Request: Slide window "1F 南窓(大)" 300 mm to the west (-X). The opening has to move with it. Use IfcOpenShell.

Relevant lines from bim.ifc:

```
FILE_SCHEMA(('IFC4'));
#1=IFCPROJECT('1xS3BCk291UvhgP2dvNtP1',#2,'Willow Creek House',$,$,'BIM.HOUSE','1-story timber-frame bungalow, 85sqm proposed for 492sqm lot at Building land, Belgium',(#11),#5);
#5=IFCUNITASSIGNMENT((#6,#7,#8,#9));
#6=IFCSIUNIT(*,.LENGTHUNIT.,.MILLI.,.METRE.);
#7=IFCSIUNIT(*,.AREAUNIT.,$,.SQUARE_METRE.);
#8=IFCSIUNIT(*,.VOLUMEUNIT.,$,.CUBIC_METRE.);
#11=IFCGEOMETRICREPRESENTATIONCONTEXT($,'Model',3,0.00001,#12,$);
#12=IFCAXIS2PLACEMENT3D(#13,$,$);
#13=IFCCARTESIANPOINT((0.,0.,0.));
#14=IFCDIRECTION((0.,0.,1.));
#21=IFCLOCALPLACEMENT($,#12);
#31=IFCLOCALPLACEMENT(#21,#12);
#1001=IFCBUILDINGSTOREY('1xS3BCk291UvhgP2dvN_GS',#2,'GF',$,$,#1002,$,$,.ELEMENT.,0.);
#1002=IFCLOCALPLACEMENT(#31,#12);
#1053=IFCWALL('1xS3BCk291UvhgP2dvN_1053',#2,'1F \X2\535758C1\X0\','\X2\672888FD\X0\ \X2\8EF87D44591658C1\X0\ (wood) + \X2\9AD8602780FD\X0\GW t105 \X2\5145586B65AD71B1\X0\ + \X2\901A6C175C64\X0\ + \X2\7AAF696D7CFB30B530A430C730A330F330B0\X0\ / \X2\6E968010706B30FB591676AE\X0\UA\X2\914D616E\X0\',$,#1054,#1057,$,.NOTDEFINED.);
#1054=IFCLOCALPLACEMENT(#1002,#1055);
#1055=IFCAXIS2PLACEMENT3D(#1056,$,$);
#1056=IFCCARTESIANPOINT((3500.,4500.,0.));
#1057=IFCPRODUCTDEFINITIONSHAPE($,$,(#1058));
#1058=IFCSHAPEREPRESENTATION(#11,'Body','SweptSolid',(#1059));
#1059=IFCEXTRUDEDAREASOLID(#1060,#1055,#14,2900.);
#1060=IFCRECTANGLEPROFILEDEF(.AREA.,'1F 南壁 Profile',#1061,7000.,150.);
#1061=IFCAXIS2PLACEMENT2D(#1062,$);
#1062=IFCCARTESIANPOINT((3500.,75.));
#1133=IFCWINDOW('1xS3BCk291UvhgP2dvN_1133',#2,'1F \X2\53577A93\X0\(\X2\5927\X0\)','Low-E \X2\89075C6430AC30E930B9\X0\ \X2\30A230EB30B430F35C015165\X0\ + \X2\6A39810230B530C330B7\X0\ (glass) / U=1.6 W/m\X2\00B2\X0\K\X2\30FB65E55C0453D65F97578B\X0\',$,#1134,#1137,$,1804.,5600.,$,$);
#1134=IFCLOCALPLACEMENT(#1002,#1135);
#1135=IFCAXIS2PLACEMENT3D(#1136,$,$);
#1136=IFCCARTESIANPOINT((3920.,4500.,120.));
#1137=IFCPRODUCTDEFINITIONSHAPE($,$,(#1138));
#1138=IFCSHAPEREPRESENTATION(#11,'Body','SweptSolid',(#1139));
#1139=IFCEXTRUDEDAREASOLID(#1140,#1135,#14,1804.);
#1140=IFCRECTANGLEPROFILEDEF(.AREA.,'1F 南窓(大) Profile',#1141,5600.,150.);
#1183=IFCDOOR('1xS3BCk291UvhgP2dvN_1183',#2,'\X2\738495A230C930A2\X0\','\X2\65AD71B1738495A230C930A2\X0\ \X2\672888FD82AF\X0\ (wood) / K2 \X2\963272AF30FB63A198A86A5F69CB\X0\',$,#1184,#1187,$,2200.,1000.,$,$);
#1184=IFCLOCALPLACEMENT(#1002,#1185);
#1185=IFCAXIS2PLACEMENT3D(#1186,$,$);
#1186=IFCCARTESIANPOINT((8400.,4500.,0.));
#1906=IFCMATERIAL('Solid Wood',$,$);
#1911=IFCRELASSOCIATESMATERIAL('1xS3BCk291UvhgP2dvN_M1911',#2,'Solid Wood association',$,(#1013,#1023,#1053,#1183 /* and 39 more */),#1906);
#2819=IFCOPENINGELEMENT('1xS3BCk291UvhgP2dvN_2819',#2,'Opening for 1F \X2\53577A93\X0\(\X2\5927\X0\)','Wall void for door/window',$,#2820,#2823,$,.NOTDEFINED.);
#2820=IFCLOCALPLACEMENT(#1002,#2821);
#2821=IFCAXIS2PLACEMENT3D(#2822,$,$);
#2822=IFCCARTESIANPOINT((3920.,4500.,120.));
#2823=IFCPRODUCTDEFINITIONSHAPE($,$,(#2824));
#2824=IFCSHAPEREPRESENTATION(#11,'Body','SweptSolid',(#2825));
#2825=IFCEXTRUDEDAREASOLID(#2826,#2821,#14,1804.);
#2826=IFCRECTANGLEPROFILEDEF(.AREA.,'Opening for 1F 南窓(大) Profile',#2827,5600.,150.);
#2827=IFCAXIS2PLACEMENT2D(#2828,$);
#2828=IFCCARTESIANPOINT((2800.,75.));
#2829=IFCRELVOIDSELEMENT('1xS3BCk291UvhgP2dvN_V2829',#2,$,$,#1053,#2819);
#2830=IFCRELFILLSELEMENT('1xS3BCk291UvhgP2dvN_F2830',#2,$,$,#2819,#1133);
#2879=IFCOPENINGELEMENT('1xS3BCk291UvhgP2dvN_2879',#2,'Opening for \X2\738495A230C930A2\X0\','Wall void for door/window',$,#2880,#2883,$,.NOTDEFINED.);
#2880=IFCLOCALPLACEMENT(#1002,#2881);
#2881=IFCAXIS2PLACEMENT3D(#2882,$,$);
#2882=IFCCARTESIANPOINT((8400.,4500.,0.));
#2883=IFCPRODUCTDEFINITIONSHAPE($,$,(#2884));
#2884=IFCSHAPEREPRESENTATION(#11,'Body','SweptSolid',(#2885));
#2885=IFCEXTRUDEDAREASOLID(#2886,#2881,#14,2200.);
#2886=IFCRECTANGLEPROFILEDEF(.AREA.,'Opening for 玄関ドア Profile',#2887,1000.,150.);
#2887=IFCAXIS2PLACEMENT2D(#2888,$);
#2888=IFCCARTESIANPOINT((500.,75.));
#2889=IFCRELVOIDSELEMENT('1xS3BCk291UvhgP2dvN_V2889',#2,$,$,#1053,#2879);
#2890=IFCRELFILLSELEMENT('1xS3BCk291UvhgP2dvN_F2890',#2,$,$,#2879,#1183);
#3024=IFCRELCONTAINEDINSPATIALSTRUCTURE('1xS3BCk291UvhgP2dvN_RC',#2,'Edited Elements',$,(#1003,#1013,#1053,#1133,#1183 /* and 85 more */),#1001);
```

```python
import ifcopenshell
import ifcopenshell.api.geometry
import ifcopenshell.util.placement
import ifcopenshell.util.unit

model = ifcopenshell.open("bim.ifc")
unit_scale = ifcopenshell.util.unit.calculate_unit_scale(model)

window = model.by_guid("1xS3BCk291UvhgP2dvN_1133")
opening = window.FillsVoids[0].RelatingOpeningElement
wall = opening.VoidsElements[0].RelatingBuildingElement

wall_matrix = ifcopenshell.util.placement.get_local_placement(wall.ObjectPlacement)
shift = wall_matrix[:3, 0] * -0.3 / unit_scale
before = ifcopenshell.util.placement.get_local_placement(window.ObjectPlacement)[:3, 3].copy()

# The window is not placed relative to its opening, so move both.
for product in (opening, window):
    matrix = ifcopenshell.util.placement.get_local_placement(product.ObjectPlacement)
    matrix[:3, 3] += shift
    ifcopenshell.api.geometry.edit_object_placement(model, product=product, matrix=matrix, is_si=False)

after = ifcopenshell.util.placement.get_local_placement(window.ObjectPlacement)[:3, 3]
print("window moved by", (after - before).round(3) + 0.0)

model.write("bim_rev.ifc")
```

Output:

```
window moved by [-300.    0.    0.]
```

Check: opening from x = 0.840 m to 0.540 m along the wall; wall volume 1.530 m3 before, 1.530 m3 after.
